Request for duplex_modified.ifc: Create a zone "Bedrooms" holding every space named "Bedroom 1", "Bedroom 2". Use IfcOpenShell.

First a look at what the model holds.

```python
import ifcopenshell

model = ifcopenshell.open("duplex_modified.ifc")
print(model.schema)
seen = {}
for space in model.by_type("IfcSpace"):
    seen[space.LongName] = seen.get(space.LongName, 0) + 1
for name, count in sorted(seen.items(), key=str):
    print(count, "x", name)
print("zones:", [z.Name for z in model.by_type("IfcZone")][:20])
```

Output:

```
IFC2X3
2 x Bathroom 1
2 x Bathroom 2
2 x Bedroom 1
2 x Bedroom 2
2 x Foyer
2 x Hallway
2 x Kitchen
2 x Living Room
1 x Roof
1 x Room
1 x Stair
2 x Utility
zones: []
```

```python
import ifcopenshell
import ifcopenshell.api.group
import ifcopenshell.api.root

model = ifcopenshell.open("duplex_modified.ifc")

names = {"Bedroom 1", "Bedroom 2"}
spaces = [s for s in model.by_type("IfcSpace") if s.LongName in names]

zone = ifcopenshell.api.root.create_entity(model, ifc_class="IfcZone", name="Bedrooms")
ifcopenshell.api.group.assign_group(model, products=spaces, group=zone)
print(len(spaces), "spaces in", zone.Name)

model.write("duplex_modified_v2.ifc")
```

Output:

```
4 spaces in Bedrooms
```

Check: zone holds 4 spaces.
